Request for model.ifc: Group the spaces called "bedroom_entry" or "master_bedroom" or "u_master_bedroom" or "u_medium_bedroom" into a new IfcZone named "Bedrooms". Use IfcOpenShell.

First a look at what the model holds.

```python
import ifcopenshell

model = ifcopenshell.open("model.ifc")
print(model.schema)
seen = {}
for space in model.by_type("IfcSpace"):
    seen[space.LongName] = seen.get(space.LongName, 0) + 1
for name, count in sorted(seen.items(), key=str):
    print(count, "x", name)
print("zones:", [z.Name for z in model.by_type("IfcZone")][:20])
```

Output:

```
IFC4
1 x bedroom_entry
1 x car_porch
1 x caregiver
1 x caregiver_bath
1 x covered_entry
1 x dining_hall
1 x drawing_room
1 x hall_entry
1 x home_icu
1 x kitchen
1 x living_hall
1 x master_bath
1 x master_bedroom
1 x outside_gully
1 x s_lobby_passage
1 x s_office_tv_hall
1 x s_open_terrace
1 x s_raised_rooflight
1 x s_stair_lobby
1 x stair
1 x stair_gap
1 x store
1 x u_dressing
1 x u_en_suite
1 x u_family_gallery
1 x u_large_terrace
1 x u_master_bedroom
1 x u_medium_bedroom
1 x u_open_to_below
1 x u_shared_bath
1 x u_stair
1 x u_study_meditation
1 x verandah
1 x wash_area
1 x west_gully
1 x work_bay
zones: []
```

```python
import ifcopenshell
import ifcopenshell.api.group
import ifcopenshell.api.root

model = ifcopenshell.open("model.ifc")

names = {"bedroom_entry", "master_bedroom", "u_master_bedroom", "u_medium_bedroom"}
spaces = [s for s in model.by_type("IfcSpace") if s.LongName in names]

zone = ifcopenshell.api.root.create_entity(model, ifc_class="IfcZone", name="Bedrooms")
ifcopenshell.api.group.assign_group(model, products=spaces, group=zone)
print(len(spaces), "spaces in", zone.Name)

model.write("model-out.ifc")
```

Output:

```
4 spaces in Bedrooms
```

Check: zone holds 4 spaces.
